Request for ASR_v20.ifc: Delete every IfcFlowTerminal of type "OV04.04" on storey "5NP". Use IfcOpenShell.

First a look at what the model holds.

```python
import ifcopenshell
import ifcopenshell.util.element

model = ifcopenshell.open("ASR_v20.ifc")
print(model.schema)
storey = next(s for s in model.by_type("IfcBuildingStorey") if s.Name == "5NP")
terminals = [e for e in ifcopenshell.util.element.get_decomposition(storey) if e.is_a("IfcFlowTerminal")]
seen = {}
for e in terminals:
    element_type = ifcopenshell.util.element.get_type(e)
    name = element_type.Name if element_type not in (None, e) else None
    seen[name] = seen.get(name, 0) + 1
for name, count in sorted(seen.items(), key=str):
    print(count, "x", name)
```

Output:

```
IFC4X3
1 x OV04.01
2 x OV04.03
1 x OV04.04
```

```python
import ifcopenshell
import ifcopenshell.api.root
import ifcopenshell.util.element

model = ifcopenshell.open("ASR_v20.ifc")

storey = next(s for s in model.by_type("IfcBuildingStorey") if s.Name == "5NP")
terminals = [e for e in ifcopenshell.util.element.get_decomposition(storey) if e.is_a("IfcFlowTerminal")]
targets = [e for e in terminals if (t := ifcopenshell.util.element.get_type(e)) not in (None, e) and t.Name == "OV04.04"]

for e in targets:
    ifcopenshell.api.root.remove_product(model, product=e)
print(len(targets), "removed")

model.write("ASR_v20_v2.ifc")
```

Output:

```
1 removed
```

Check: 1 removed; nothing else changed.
